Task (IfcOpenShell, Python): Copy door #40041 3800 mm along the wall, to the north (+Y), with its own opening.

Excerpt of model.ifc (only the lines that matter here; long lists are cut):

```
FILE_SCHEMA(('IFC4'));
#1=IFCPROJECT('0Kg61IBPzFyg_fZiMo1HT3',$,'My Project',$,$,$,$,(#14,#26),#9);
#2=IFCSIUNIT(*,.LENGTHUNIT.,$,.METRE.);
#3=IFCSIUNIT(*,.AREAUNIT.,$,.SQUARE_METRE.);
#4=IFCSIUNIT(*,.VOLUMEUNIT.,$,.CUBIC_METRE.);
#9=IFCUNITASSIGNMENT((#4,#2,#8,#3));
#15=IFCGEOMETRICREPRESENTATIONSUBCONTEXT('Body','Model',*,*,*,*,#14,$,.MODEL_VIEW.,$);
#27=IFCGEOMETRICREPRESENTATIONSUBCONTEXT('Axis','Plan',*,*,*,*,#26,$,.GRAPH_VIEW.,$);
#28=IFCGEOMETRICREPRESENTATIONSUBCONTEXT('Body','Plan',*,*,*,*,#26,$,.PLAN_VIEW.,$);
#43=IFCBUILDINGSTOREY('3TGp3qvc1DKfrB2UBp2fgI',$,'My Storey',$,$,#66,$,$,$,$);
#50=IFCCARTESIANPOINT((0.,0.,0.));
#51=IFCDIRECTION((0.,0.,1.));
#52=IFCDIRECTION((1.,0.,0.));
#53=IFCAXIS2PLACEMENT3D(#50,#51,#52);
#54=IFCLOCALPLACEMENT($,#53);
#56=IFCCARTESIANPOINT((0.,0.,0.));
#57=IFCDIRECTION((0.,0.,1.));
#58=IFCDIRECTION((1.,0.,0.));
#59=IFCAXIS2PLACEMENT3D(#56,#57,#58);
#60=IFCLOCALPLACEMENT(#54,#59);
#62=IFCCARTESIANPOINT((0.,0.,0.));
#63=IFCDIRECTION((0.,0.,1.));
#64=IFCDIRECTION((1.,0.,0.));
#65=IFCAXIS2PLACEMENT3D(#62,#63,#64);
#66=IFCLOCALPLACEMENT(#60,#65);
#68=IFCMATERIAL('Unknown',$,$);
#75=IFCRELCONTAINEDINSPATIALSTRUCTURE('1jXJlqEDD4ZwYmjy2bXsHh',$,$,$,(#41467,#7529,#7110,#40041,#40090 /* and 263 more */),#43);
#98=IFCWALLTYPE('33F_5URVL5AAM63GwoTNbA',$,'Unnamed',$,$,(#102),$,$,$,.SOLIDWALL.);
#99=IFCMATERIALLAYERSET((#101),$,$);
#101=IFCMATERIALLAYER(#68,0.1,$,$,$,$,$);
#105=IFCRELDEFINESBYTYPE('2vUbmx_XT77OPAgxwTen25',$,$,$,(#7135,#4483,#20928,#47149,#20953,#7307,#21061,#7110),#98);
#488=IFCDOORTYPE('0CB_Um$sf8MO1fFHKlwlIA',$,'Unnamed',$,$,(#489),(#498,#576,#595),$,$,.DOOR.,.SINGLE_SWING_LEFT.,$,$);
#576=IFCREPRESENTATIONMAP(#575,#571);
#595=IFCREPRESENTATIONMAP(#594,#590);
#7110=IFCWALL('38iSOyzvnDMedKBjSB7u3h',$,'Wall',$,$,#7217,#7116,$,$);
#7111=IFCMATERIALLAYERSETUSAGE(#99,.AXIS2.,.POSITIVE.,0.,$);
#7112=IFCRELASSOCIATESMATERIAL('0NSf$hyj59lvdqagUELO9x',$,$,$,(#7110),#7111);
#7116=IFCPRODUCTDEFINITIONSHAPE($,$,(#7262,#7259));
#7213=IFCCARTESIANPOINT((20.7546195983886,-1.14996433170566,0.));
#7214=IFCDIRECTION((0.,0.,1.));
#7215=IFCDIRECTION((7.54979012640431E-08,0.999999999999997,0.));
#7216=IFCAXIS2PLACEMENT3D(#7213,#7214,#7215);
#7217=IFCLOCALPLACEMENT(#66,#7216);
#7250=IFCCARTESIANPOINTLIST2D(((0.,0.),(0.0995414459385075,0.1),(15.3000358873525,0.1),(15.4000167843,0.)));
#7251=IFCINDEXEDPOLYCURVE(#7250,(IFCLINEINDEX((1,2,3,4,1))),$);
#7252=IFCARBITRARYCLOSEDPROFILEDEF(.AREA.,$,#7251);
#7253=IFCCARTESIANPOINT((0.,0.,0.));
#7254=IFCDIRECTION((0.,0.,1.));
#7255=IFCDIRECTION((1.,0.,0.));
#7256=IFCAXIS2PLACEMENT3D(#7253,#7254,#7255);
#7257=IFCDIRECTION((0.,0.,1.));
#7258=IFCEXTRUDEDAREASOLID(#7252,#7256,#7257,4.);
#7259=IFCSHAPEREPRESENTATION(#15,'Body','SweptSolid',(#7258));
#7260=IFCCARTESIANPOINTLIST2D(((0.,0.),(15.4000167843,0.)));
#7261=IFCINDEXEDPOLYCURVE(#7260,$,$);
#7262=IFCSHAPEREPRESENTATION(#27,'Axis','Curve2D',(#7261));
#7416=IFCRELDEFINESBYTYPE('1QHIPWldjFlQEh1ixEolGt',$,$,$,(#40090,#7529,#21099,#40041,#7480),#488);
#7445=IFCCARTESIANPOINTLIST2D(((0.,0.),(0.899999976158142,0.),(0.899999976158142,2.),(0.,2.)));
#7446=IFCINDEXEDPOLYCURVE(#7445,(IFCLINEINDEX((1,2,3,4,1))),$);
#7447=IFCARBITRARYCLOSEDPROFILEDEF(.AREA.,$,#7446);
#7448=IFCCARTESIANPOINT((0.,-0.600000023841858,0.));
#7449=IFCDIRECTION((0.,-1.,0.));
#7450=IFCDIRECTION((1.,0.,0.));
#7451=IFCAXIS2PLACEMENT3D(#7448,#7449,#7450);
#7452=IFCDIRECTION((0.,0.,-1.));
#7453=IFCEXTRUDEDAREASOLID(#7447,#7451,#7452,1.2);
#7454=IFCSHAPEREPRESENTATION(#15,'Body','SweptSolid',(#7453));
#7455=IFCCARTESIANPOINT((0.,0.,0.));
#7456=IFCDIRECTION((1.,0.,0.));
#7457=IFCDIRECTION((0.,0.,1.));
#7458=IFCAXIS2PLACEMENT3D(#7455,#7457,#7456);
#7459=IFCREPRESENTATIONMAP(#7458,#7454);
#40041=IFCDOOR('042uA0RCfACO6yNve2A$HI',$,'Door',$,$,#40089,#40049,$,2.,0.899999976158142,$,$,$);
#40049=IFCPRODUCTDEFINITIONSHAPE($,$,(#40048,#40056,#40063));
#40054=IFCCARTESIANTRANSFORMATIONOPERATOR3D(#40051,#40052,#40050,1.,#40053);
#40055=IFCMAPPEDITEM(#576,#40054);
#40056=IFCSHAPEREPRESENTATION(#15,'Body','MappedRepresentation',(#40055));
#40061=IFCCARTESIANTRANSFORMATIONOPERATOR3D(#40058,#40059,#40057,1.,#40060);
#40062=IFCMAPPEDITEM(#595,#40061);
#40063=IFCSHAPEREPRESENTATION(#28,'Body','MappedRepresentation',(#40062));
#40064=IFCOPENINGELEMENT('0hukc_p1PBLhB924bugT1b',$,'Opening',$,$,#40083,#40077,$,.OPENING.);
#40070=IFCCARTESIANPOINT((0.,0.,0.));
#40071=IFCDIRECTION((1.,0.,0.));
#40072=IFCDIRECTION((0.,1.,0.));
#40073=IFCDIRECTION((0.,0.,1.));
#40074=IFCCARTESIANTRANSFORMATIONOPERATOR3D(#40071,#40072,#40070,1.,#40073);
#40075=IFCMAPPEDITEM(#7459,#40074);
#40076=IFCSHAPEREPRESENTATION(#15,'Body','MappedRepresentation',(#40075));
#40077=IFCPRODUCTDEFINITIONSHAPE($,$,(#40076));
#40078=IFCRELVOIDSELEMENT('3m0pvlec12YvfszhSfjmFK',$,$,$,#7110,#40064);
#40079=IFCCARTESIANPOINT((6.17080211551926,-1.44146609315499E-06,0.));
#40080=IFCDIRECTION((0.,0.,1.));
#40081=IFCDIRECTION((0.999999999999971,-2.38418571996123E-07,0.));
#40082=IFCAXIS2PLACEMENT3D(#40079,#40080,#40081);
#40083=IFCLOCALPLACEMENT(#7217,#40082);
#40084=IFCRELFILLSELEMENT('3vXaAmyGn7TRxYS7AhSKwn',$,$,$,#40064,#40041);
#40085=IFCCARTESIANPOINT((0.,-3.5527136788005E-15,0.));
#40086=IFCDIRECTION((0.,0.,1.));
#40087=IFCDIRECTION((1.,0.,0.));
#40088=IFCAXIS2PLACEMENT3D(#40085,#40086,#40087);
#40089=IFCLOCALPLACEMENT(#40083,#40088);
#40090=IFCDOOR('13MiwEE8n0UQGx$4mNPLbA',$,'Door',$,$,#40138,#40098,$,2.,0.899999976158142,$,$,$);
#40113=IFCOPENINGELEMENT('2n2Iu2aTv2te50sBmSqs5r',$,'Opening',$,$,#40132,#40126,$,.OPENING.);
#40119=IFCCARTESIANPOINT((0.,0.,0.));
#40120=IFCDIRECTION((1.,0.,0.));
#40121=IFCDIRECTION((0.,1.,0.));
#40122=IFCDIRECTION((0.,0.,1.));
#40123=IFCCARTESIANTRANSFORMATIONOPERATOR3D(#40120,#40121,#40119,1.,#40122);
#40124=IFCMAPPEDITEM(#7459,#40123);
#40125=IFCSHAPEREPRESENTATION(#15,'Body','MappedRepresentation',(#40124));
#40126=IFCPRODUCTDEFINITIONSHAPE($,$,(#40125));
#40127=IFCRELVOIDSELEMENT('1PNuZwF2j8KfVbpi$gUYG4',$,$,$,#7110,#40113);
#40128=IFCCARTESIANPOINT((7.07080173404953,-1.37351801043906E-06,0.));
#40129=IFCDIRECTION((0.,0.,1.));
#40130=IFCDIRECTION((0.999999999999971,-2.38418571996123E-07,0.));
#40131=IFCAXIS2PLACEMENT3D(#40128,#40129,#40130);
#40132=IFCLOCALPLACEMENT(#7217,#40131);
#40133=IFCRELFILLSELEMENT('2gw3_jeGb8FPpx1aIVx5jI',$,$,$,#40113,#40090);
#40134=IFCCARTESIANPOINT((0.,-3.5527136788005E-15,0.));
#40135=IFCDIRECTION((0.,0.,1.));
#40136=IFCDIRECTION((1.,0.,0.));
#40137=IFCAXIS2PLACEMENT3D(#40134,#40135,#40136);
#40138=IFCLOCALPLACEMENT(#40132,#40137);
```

```python
import ifcopenshell
import ifcopenshell.api.feature
import ifcopenshell.api.geometry
import ifcopenshell.api.root
import ifcopenshell.geom
import ifcopenshell.util.element
import ifcopenshell.util.placement
import ifcopenshell.util.shape
import ifcopenshell.util.unit

model = ifcopenshell.open("model.ifc")
unit_scale = ifcopenshell.util.unit.calculate_unit_scale(model)
settings = ifcopenshell.geom.settings()


def volume(element):
    """Net volume in cubic metres, openings subtracted."""
    shape = ifcopenshell.geom.create_shape(settings, element)
    return ifcopenshell.util.shape.get_volume(shape.geometry)


door = model.by_id(40041)
opening = door.FillsVoids[0].RelatingOpeningElement
wall = opening.VoidsElements[0].RelatingBuildingElement
before = volume(wall)
shift = ifcopenshell.util.placement.get_local_placement(wall.ObjectPlacement)[:3, 0] * 3.8 / unit_scale

# copy_class copies the void relationship, type, container and properties, but no geometry.
new_opening = ifcopenshell.api.root.copy_class(model, product=opening)
new_opening.Representation = ifcopenshell.util.element.copy_deep(
    model, opening.Representation, exclude=["IfcGeometricRepresentationContext", "IfcRepresentationMap"]
)
new_door = ifcopenshell.api.root.copy_class(model, product=door)
new_door.Representation = ifcopenshell.util.element.copy_deep(
    model, door.Representation, exclude=["IfcGeometricRepresentationContext", "IfcRepresentationMap"]
)
ifcopenshell.api.feature.add_filling(model, opening=new_opening, element=new_door)

for old, new in ((opening, new_opening), (door, new_door)):
    matrix = ifcopenshell.util.placement.get_local_placement(old.ObjectPlacement)
    matrix[:3, 3] += shift
    ifcopenshell.api.geometry.edit_object_placement(model, product=new, matrix=matrix, is_si=False)

after = volume(wall)

print(f"wall volume {before:.3f} -> {after:.3f} m3")

model.write("model-out.ifc")
```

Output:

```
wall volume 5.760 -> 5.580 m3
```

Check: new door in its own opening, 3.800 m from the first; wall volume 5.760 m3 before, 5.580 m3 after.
